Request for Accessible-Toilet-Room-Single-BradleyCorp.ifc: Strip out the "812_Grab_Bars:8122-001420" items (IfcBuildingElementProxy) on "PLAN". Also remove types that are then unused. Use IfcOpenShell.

First a look at what the model holds.

```python
import ifcopenshell
import ifcopenshell.util.element

model = ifcopenshell.open("Accessible-Toilet-Room-Single-BradleyCorp.ifc")
print(model.schema)
storey = next(s for s in model.by_type("IfcBuildingStorey") if s.Name == "PLAN")
proxies = [e for e in ifcopenshell.util.element.get_decomposition(storey) if e.is_a("IfcBuildingElementProxy")]
seen = {}
for e in proxies:
    element_type = ifcopenshell.util.element.get_type(e)
    name = element_type.Name if element_type not in (None, e) else None
    seen[name] = seen.get(name, 0) + 1
for name, count in sorted(seen.items(), key=str):
    print(count, "x", name)
```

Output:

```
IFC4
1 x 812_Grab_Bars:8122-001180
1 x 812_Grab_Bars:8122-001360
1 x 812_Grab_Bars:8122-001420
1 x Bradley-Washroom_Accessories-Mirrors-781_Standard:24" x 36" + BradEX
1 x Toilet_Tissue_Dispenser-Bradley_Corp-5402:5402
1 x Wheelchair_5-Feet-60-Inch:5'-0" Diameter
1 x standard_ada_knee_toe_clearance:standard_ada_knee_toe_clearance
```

```python
import ifcopenshell
import ifcopenshell.api.root
import ifcopenshell.util.element

model = ifcopenshell.open("Accessible-Toilet-Room-Single-BradleyCorp.ifc")

storey = next(s for s in model.by_type("IfcBuildingStorey") if s.Name == "PLAN")
proxies = [e for e in ifcopenshell.util.element.get_decomposition(storey) if e.is_a("IfcBuildingElementProxy")]
targets = [e for e in proxies if (t := ifcopenshell.util.element.get_type(e)) not in (None, e) and t.Name == "812_Grab_Bars:8122-001420"]
types = {ifcopenshell.util.element.get_type(e) for e in targets} - {None, *targets}

for e in targets:
    ifcopenshell.api.root.remove_product(model, product=e)
print(len(targets), "removed")

unused = [t for t in types if not ifcopenshell.util.element.get_types(t)]
for t in unused:
    ifcopenshell.api.root.remove_product(model, product=t)
print(len(unused), "unused types removed")

model.write("Accessible-Toilet-Room-Single-BradleyCorp_edited.ifc")
```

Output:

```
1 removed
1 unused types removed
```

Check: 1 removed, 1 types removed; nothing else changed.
